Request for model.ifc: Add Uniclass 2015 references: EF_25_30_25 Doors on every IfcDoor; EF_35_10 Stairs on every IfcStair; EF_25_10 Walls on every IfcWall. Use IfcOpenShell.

First a look at what the model holds.

```python
import ifcopenshell

model = ifcopenshell.open("model.ifc")
print(model.schema)
print("classifications:", [c.Name for c in model.by_type("IfcClassification")])
for ifc_class in ("IfcDoor", "IfcRoof", "IfcStair", "IfcWall", "IfcWindow"):
    print(ifc_class, len(model.by_type(ifc_class)))
```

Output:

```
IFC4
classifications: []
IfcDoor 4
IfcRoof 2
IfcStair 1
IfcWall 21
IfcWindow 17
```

```python
import ifcopenshell
import ifcopenshell.api.classification

model = ifcopenshell.open("model.ifc")

system = ifcopenshell.api.classification.add_classification(model, classification="Uniclass 2015")

codes = {
    "IfcDoor": ("EF_25_30_25", "Doors"),
    "IfcStair": ("EF_35_10", "Stairs"),
    "IfcWall": ("EF_25_10", "Walls"),
}
for ifc_class, (code, name) in codes.items():
    products = model.by_type(ifc_class)
    ifcopenshell.api.classification.add_reference(
        model, products=products, classification=system, identification=code, name=name
    )
    print(code, len(products))

model.write("model_updated.ifc")
```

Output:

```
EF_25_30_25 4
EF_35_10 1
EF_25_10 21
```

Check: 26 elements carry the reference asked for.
